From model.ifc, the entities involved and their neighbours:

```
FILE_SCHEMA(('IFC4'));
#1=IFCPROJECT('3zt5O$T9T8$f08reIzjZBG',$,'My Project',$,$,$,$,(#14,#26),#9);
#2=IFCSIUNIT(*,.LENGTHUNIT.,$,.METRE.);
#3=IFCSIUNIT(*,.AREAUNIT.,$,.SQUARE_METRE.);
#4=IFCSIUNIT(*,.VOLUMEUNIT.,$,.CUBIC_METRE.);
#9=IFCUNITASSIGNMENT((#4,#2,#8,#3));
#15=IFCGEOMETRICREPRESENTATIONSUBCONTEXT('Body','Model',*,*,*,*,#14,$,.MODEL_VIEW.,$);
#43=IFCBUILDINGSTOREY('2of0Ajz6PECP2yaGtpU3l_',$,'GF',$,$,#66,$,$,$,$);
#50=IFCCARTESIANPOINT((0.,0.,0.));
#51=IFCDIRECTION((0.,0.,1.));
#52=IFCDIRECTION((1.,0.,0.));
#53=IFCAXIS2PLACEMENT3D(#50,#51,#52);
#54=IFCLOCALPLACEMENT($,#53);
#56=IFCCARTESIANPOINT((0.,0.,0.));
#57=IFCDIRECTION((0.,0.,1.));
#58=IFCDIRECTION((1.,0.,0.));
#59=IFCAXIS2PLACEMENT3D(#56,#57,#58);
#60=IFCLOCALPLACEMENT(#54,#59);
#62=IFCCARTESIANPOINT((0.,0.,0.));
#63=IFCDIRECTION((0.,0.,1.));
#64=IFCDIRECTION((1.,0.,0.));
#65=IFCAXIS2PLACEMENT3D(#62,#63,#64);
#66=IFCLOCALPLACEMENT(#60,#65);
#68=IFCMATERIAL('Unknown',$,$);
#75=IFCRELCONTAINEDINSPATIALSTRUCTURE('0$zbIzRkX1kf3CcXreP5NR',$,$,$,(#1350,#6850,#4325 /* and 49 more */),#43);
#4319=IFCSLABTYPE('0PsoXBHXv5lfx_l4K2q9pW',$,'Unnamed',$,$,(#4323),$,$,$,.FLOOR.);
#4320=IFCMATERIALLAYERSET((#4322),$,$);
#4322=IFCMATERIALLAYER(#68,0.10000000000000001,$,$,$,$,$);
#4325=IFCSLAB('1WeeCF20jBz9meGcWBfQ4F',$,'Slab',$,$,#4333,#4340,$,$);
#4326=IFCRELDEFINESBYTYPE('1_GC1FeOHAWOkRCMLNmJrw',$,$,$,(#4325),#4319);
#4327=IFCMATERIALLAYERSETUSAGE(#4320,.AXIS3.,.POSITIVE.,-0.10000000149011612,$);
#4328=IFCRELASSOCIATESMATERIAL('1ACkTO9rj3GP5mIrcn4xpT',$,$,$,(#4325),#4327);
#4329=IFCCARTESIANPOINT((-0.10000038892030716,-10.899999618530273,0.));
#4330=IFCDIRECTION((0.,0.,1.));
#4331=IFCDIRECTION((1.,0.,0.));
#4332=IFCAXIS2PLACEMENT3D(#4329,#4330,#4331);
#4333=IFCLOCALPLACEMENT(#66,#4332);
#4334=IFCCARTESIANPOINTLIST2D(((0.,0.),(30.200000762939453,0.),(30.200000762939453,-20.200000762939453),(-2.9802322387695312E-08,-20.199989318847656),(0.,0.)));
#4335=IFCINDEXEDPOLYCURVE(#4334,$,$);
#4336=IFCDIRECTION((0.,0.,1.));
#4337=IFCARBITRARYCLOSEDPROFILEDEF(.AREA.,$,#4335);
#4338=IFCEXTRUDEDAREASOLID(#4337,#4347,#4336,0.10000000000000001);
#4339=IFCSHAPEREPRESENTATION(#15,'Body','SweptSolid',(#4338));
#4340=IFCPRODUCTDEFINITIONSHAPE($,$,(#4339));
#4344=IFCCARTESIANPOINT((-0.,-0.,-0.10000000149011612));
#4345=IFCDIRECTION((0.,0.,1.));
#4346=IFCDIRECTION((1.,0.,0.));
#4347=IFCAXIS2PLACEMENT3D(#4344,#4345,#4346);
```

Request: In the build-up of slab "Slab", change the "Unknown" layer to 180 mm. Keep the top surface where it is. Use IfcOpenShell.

```python
import ifcopenshell
import ifcopenshell.util.element
import ifcopenshell.util.representation
import ifcopenshell.util.unit

model = ifcopenshell.open("model.ifc")
unit_scale = ifcopenshell.util.unit.calculate_unit_scale(model)

layer_set = model.by_id(4320)
layer = next(l for l in layer_set.MaterialLayers if l.Material and l.Material.Name == "Unknown")
change = 0.18 / unit_scale - layer.LayerThickness
layer.LayerThickness += change

# Geometry does not follow the layer set by itself.
slabs = [e for e in ifcopenshell.util.element.get_elements_by_material(model, layer_set) if e.is_a("IfcSlab")]
for slab in sorted(slabs, key=lambda e: e.id()):
    body = ifcopenshell.util.representation.get_representation(slab, "Model", "Body")
    solid = body.Items[0]
    old_depth = solid.Depth
    solid.Depth += change
    # Extruded upwards: lower the start of the extrusion so the top stays.
    x, y, z = solid.Position.Location.Coordinates
    solid.Position.Location = model.createIfcCartesianPoint((x, y, z - change))
    print(slab.id(), f"{old_depth:g} -> {solid.Depth:g}")

# The layers are counted up from the underside, which has moved.
for usage in {ifcopenshell.util.element.get_material(slab) for slab in slabs}:
    usage.OffsetFromReferenceLine -= change

model.write("model_updated.ifc")
```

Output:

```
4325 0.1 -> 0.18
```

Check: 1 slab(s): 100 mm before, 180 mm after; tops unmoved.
